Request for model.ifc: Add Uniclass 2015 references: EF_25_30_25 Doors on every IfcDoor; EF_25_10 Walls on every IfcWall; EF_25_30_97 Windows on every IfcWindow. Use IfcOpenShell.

First a look at what the model holds.

```python
import ifcopenshell

model = ifcopenshell.open("model.ifc")
print(model.schema)
print("classifications:", [c.Name for c in model.by_type("IfcClassification")])
for ifc_class in ("IfcDoor", "IfcRoof", "IfcStair", "IfcWall", "IfcWindow"):
    print(ifc_class, len(model.by_type(ifc_class)))
```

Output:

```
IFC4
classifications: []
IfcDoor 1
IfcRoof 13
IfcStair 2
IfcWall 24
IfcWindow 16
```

```python
import ifcopenshell
import ifcopenshell.api.classification

model = ifcopenshell.open("model.ifc")

system = ifcopenshell.api.classification.add_classification(model, classification="Uniclass 2015")

codes = {
    "IfcDoor": ("EF_25_30_25", "Doors"),
    "IfcWall": ("EF_25_10", "Walls"),
    "IfcWindow": ("EF_25_30_97", "Windows"),
}
for ifc_class, (code, name) in codes.items():
    products = model.by_type(ifc_class)
    ifcopenshell.api.classification.add_reference(
        model, products=products, classification=system, identification=code, name=name
    )
    print(code, len(products))

model.write("model-out.ifc")
```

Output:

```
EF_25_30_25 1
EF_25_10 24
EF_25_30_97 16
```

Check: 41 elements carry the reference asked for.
